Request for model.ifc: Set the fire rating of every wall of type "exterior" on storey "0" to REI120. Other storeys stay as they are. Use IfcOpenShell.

First a look at what the model holds.

```python
import ifcopenshell
import ifcopenshell.util.element

model = ifcopenshell.open("model.ifc")
print(model.schema)
storey = next(s for s in model.by_type("IfcBuildingStorey") if s.Name == "0")
walls = [e for e in ifcopenshell.util.element.get_decomposition(storey) if e.is_a("IfcWall")]
seen = {}
for e in walls:
    element_type = ifcopenshell.util.element.get_type(e)
    key = (element_type.Name if element_type != e and element_type else None, ifcopenshell.util.element.get_pset(e, "Pset_WallCommon", "FireRating"))
    seen[key] = seen.get(key, 0) + 1
for (name, value), count in sorted(seen.items(), key=str):
    print(count, "x", name, "|", value)
```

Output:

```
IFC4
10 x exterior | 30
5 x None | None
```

```python
import ifcopenshell
import ifcopenshell.api.pset
import ifcopenshell.util.element

model = ifcopenshell.open("model.ifc")

storey = next(s for s in model.by_type("IfcBuildingStorey") if s.Name == "0")
walls = [e for e in ifcopenshell.util.element.get_decomposition(storey) if e.is_a("IfcWall")]

count = 0
for e in walls:
    element_type = ifcopenshell.util.element.get_type(e)
    if element_type in (None, e) or element_type.Name != "exterior":
        continue
    # add_pset returns the element's existing set when there is one.
    pset = ifcopenshell.api.pset.add_pset(model, product=e, name="Pset_WallCommon")
    ifcopenshell.api.pset.edit_pset(model, pset=pset, properties={"FireRating": "REI120"})
    count += 1

print(count, "walls updated")

model.write("model_edited.ifc")
```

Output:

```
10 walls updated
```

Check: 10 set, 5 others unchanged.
